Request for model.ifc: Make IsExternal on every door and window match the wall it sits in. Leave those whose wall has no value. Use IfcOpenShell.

First a look at what the model holds.

```python
import ifcopenshell
import ifcopenshell.util.element

model = ifcopenshell.open("model.ifc")
print(model.schema)
seen = {}
for e in model.by_type("IfcDoor") + model.by_type("IfcWindow"):
    if not e.FillsVoids:
        continue
    host = e.FillsVoids[0].RelatingOpeningElement.VoidsElements[0].RelatingBuildingElement
    own = ifcopenshell.util.element.get_pset(e, f"Pset_{e.is_a()[3:].removesuffix('StandardCase')}Common", "IsExternal")
    wall = ifcopenshell.util.element.get_pset(host, "Pset_WallCommon", "IsExternal")
    seen[e.is_a(), own, wall] = seen.get((e.is_a(), own, wall), 0) + 1
for (cls, own, wall), count in sorted(seen.items(), key=str):
    print(count, cls, "IsExternal:", own, "| host wall:", wall)
```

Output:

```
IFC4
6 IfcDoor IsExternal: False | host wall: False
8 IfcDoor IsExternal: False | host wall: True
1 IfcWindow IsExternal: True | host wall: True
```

```python
import ifcopenshell
import ifcopenshell.api.pset
import ifcopenshell.util.element

model = ifcopenshell.open("model.ifc")

count = 0
for ifc_class, pset_name in (("IfcDoor", "Pset_DoorCommon"), ("IfcWindow", "Pset_WindowCommon")):
    for e in model.by_type(ifc_class):
        if not e.FillsVoids:
            continue
        host = e.FillsVoids[0].RelatingOpeningElement.VoidsElements[0].RelatingBuildingElement
        external = ifcopenshell.util.element.get_pset(host, "Pset_WallCommon", "IsExternal")
        if external is None or ifcopenshell.util.element.get_pset(e, pset_name, "IsExternal") == external:
            continue
        pset = ifcopenshell.api.pset.add_pset(model, product=e, name=pset_name)
        ifcopenshell.api.pset.edit_pset(model, pset=pset, properties={"IsExternal": external})
        count += 1

print(count, "updated")

model.write("model-out.ifc")
```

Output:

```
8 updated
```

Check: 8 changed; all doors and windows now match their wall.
